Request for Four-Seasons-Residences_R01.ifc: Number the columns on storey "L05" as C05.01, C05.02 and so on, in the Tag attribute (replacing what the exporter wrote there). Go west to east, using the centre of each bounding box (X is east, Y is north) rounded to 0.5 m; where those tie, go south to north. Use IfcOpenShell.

First a look at what the model holds.

```python
import ifcopenshell
import ifcopenshell.util.element
import ifcopenshell.util.placement

model = ifcopenshell.open("Four-Seasons-Residences_R01.ifc")
print(model.schema)
storey = next(s for s in model.by_type("IfcBuildingStorey") if s.Name == "L05")
columns = [e for e in ifcopenshell.util.element.get_decomposition(storey) if e.is_a("IfcColumn")]
for e in sorted(columns, key=lambda e: e.id()):
    origin = ifcopenshell.util.placement.get_local_placement(e.ObjectPlacement)[:3, 3]
    print(e.id(), e.Tag, e.Name, origin.round(2) + 0.0, sep=" | ")
```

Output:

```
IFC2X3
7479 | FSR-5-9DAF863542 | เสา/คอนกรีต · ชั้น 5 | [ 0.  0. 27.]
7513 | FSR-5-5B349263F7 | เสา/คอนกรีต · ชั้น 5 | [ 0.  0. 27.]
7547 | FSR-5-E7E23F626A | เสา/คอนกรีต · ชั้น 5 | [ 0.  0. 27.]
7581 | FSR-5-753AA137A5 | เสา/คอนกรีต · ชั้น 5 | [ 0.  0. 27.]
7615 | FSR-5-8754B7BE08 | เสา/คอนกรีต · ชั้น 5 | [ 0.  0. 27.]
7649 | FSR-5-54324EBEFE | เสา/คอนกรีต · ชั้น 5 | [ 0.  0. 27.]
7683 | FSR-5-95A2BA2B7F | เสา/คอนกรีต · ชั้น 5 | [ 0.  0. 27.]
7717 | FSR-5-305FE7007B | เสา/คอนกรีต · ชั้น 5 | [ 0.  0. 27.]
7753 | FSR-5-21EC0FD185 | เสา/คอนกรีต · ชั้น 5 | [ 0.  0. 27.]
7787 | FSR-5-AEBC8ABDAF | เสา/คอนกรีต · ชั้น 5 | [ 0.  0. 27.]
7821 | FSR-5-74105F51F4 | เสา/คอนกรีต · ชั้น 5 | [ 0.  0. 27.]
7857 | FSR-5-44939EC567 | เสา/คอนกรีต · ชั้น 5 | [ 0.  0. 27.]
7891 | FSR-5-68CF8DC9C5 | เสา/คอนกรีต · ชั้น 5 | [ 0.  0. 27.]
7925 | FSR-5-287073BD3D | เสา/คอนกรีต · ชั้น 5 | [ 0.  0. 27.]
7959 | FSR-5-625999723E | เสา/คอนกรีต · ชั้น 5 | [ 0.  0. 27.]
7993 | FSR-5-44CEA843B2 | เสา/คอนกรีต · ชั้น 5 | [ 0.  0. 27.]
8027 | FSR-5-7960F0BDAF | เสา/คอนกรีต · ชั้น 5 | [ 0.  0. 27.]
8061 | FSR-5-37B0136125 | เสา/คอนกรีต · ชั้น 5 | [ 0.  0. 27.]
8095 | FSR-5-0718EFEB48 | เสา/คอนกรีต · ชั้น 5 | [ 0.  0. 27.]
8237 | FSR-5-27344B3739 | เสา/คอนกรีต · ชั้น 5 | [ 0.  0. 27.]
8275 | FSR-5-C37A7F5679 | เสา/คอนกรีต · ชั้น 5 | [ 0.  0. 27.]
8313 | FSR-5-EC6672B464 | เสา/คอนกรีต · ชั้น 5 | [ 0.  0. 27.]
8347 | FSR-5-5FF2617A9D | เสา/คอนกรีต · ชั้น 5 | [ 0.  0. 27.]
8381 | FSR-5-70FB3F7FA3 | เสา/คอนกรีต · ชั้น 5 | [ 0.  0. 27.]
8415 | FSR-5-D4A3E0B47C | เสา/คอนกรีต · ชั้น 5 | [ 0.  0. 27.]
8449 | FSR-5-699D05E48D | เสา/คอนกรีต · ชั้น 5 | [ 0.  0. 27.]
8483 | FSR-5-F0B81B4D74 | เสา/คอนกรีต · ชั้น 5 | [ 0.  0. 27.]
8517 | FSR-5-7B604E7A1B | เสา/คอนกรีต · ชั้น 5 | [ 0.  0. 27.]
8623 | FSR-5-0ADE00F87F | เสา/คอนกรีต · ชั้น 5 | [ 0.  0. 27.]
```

```python
import ifcopenshell
import ifcopenshell.geom
import ifcopenshell.util.element
import ifcopenshell.util.shape

model = ifcopenshell.open("Four-Seasons-Residences_R01.ifc")
settings = ifcopenshell.geom.settings()
settings.set("use-world-coords", True)


def centre(element):
    shape = ifcopenshell.geom.create_shape(settings, element)
    return ifcopenshell.util.shape.get_bbox_centroid(shape.geometry)


storey = next(s for s in model.by_type("IfcBuildingStorey") if s.Name == "L05")
columns = [e for e in ifcopenshell.util.element.get_decomposition(storey) if e.is_a("IfcColumn")]

# Insertion points can sit at a corner or the storey origin, so sort by the geometry (in metres).
centres = {e: centre(e) for e in columns}
columns.sort(key=lambda e: (round(centres[e][0] / 0.5), centres[e][1]))

for i, e in enumerate(columns, start=1):
    number = f"C05.{i:02d}"
    e.Tag = number
    print(e.id(), number)

model.write("Four-Seasons-Residences_R01_rev.ifc")
```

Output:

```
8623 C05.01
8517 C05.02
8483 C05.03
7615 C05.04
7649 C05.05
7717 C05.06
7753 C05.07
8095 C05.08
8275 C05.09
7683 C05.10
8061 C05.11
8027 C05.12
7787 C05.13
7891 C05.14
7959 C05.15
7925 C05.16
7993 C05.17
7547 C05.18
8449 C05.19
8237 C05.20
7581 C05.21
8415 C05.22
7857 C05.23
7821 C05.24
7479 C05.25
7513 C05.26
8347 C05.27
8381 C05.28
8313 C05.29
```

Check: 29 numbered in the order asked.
